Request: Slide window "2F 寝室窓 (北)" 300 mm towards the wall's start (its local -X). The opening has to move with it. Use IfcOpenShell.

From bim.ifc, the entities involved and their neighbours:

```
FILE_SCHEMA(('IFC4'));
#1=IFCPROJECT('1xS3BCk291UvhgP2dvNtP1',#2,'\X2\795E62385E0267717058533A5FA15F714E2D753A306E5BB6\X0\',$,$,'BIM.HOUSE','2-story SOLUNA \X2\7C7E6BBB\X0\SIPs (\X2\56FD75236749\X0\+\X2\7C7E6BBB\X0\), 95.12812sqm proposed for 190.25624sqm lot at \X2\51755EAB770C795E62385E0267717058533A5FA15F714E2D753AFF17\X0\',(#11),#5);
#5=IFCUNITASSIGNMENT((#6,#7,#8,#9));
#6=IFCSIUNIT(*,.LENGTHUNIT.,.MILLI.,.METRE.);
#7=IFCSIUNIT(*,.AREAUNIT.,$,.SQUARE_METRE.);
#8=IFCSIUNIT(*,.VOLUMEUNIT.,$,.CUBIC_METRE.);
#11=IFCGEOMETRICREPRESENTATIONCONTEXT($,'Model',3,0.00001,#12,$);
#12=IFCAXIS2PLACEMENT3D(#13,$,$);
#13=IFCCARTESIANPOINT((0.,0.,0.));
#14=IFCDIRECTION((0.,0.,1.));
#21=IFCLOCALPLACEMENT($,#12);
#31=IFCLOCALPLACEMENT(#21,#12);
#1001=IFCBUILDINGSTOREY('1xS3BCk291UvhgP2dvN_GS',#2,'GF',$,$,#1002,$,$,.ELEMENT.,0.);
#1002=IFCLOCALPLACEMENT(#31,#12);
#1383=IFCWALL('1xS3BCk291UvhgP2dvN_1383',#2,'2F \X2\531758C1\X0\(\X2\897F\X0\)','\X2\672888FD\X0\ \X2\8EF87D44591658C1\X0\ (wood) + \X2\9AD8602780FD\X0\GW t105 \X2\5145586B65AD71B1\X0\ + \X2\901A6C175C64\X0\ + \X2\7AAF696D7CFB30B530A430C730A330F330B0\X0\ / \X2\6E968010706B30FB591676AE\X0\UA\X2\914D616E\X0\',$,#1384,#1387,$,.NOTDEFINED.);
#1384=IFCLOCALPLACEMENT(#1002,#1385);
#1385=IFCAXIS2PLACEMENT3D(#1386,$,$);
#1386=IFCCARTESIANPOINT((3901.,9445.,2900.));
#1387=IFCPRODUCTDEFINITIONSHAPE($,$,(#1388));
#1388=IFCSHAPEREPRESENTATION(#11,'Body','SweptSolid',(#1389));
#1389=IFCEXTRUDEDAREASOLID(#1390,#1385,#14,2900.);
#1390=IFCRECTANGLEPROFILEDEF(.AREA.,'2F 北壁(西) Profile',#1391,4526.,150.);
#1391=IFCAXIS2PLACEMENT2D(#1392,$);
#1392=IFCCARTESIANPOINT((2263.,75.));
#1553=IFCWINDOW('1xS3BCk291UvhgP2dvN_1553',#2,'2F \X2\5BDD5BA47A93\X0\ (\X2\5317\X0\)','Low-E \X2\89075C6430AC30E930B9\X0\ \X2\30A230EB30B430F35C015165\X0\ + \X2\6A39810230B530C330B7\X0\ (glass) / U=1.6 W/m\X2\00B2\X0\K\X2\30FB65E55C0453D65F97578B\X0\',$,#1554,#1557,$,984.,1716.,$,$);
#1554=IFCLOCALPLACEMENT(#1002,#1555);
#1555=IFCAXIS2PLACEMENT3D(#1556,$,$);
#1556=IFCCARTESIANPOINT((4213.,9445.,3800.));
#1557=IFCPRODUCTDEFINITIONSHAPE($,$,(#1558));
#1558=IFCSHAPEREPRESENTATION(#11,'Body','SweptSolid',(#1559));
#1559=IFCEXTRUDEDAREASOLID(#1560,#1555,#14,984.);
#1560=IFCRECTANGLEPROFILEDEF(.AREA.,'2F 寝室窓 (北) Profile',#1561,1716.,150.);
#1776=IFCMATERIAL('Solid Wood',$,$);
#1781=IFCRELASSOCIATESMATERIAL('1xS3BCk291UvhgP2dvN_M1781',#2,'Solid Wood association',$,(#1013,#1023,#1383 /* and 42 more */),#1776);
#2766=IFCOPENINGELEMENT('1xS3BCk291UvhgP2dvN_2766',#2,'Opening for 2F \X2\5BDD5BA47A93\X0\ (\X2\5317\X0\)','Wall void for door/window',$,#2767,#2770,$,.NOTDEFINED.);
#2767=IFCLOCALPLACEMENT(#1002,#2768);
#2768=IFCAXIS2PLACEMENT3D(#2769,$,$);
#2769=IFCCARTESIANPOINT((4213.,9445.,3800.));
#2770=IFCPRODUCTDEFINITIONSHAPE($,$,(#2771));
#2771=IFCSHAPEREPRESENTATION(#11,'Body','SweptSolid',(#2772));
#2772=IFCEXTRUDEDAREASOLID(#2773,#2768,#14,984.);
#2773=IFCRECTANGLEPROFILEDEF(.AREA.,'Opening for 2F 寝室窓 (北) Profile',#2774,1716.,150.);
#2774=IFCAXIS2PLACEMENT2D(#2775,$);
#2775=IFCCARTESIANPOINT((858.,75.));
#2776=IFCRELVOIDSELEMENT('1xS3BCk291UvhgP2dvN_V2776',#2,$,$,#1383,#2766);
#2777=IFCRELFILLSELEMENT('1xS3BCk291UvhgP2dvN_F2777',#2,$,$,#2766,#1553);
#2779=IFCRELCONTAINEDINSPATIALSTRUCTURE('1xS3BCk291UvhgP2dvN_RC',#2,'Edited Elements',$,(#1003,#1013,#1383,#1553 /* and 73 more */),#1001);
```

```python
import ifcopenshell
import ifcopenshell.api.geometry
import ifcopenshell.util.placement
import ifcopenshell.util.unit

model = ifcopenshell.open("bim.ifc")
unit_scale = ifcopenshell.util.unit.calculate_unit_scale(model)

window = model.by_id(1553)
opening = window.FillsVoids[0].RelatingOpeningElement
wall = opening.VoidsElements[0].RelatingBuildingElement

wall_matrix = ifcopenshell.util.placement.get_local_placement(wall.ObjectPlacement)
shift = wall_matrix[:3, 0] * -0.3 / unit_scale
before = ifcopenshell.util.placement.get_local_placement(window.ObjectPlacement)[:3, 3].copy()

# The window is not placed relative to its opening, so move both.
for product in (opening, window):
    matrix = ifcopenshell.util.placement.get_local_placement(product.ObjectPlacement)
    matrix[:3, 3] += shift
    ifcopenshell.api.geometry.edit_object_placement(model, product=product, matrix=matrix, is_si=False)

after = ifcopenshell.util.placement.get_local_placement(window.ObjectPlacement)[:3, 3]
print("window moved by", (after - before).round(3) + 0.0)

model.write("bim_rev.ifc")
```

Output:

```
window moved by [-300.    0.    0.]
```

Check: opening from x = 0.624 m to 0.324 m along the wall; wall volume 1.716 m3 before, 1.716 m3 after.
